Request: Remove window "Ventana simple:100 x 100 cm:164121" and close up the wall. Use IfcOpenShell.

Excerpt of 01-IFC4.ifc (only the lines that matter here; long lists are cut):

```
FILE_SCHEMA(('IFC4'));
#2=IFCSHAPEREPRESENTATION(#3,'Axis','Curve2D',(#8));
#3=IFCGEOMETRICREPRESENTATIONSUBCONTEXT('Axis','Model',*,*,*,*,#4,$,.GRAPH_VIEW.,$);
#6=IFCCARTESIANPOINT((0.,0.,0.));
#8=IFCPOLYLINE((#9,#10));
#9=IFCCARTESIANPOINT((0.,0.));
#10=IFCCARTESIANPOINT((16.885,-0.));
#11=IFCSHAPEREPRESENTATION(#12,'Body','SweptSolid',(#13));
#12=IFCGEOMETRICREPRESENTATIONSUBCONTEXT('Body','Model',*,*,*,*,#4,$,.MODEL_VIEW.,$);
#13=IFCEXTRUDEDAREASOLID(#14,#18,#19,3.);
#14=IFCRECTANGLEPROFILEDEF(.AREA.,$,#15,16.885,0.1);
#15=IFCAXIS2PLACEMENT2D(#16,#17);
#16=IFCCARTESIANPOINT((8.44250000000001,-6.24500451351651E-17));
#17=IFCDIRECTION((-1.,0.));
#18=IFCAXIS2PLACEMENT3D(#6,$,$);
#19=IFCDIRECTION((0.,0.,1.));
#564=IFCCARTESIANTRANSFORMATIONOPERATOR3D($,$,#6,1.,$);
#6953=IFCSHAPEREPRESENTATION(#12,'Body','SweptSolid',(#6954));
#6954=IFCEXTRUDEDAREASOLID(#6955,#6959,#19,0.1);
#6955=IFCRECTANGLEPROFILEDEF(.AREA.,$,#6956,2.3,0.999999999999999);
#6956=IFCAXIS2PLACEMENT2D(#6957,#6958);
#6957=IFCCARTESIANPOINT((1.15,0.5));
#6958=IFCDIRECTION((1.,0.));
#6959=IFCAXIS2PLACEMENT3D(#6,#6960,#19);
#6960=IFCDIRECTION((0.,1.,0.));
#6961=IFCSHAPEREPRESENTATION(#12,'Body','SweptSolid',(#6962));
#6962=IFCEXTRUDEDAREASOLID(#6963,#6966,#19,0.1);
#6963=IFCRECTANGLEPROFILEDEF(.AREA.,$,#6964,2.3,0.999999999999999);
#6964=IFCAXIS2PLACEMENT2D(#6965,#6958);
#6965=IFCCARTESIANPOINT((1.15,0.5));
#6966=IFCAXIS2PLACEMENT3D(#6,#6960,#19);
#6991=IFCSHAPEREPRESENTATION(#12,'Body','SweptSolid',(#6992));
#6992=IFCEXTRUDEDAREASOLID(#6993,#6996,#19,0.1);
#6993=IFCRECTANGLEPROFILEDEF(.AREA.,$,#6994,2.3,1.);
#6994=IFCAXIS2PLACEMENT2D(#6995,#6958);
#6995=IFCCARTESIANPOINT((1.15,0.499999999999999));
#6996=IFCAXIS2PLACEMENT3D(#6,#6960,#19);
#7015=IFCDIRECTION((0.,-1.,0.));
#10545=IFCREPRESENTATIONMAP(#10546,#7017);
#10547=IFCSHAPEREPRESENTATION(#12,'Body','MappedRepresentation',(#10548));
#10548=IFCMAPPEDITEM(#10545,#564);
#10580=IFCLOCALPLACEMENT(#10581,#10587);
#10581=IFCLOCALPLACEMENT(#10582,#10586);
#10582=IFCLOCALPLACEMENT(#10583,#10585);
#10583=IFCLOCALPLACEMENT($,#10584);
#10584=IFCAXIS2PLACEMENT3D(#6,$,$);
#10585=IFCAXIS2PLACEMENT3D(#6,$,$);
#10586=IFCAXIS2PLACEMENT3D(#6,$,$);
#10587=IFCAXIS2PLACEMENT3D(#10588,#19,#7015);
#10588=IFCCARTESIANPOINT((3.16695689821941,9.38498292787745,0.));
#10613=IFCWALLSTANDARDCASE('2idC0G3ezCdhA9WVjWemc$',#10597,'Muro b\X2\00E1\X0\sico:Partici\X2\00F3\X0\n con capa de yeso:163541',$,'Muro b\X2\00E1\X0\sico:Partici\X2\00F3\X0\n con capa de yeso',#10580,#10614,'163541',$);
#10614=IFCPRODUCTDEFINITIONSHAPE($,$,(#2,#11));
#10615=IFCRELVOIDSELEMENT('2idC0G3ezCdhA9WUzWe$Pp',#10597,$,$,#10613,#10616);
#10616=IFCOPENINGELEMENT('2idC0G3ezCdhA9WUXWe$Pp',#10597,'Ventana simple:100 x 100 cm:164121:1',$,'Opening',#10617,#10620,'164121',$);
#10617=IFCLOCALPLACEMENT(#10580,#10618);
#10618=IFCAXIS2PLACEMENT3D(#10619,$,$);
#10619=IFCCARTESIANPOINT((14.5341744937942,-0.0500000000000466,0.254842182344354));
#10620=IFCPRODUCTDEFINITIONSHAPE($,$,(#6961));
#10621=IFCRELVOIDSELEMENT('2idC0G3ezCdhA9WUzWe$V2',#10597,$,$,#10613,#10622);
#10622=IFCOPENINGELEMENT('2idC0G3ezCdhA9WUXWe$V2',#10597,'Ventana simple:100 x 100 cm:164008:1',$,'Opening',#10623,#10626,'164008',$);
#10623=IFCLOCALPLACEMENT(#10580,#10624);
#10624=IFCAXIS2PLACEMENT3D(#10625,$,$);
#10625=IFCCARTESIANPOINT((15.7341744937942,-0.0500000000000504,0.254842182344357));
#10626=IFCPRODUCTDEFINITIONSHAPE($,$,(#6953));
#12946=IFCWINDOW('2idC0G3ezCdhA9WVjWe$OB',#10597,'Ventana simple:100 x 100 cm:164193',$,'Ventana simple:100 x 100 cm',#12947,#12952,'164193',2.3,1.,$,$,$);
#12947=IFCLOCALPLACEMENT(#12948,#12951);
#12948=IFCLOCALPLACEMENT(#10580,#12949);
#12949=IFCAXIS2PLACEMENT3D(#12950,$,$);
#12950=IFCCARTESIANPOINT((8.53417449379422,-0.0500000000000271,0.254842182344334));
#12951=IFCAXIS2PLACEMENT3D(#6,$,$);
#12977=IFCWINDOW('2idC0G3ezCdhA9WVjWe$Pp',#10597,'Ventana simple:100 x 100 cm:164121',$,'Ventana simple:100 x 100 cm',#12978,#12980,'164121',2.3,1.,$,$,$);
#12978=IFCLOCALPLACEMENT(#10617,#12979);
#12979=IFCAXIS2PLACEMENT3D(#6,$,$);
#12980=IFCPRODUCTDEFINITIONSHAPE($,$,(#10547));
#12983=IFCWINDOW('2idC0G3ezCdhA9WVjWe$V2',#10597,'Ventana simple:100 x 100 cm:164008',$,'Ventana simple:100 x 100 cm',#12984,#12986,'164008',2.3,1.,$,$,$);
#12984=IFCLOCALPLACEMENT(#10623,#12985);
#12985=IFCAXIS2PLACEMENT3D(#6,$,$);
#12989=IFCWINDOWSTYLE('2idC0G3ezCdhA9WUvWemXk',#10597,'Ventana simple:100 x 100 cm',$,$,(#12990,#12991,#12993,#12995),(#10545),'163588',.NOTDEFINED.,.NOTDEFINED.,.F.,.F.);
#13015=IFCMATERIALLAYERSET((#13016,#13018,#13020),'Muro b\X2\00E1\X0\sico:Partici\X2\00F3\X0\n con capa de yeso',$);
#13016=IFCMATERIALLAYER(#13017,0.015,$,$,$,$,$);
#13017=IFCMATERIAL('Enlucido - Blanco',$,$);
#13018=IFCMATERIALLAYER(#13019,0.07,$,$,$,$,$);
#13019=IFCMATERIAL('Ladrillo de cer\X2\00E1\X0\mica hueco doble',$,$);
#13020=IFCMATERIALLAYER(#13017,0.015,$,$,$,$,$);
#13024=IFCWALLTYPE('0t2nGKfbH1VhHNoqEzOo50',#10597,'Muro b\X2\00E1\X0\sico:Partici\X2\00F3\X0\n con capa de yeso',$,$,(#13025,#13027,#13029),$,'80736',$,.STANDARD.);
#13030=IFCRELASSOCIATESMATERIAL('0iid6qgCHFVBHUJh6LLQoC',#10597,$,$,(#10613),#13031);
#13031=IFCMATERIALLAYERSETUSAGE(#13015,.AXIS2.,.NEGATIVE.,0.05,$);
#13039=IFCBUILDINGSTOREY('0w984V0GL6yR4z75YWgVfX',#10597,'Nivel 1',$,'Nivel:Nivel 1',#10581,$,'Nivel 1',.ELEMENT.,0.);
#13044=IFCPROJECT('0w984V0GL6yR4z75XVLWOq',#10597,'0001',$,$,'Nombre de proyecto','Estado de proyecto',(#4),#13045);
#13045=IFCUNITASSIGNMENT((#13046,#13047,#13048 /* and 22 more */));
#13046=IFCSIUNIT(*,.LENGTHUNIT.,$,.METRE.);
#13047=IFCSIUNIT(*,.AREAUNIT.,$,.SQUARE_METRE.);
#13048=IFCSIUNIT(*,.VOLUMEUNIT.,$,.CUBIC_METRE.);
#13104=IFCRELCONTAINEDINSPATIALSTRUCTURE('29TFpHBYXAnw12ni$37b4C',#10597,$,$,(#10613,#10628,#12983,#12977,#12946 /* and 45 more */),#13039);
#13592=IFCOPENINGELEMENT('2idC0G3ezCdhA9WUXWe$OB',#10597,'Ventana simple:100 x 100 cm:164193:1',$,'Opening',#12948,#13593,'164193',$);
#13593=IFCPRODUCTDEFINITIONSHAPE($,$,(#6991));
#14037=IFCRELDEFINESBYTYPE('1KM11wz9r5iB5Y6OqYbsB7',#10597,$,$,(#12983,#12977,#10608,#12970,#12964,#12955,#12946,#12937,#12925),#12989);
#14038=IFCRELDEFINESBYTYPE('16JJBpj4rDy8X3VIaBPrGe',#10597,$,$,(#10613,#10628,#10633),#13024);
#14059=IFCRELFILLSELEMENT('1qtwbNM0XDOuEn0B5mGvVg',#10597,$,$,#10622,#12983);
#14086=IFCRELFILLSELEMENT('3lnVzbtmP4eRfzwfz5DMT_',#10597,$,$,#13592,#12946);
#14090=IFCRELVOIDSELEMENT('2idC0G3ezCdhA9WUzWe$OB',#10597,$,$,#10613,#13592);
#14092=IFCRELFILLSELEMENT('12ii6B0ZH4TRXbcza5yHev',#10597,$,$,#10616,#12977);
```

```python
import ifcopenshell
import ifcopenshell.api.feature
import ifcopenshell.api.root
import ifcopenshell.geom
import ifcopenshell.util.shape

model = ifcopenshell.open("01-IFC4.ifc")
settings = ifcopenshell.geom.settings()


def volume(element):
    """Net volume in cubic metres, openings subtracted."""
    shape = ifcopenshell.geom.create_shape(settings, element)
    return ifcopenshell.util.shape.get_volume(shape.geometry)


window = model.by_id(12977)
opening = window.FillsVoids[0].RelatingOpeningElement
wall = opening.VoidsElements[0].RelatingBuildingElement
before = volume(wall)

ifcopenshell.api.root.remove_product(model, product=window)
ifcopenshell.api.feature.remove_feature(model, feature=opening)

after = volume(wall)

print(f"wall volume {before:.3f} -> {after:.3f} m3")

model.write("01-IFC4_updated.ifc")
```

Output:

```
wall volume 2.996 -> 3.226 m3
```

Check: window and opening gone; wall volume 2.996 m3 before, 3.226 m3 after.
